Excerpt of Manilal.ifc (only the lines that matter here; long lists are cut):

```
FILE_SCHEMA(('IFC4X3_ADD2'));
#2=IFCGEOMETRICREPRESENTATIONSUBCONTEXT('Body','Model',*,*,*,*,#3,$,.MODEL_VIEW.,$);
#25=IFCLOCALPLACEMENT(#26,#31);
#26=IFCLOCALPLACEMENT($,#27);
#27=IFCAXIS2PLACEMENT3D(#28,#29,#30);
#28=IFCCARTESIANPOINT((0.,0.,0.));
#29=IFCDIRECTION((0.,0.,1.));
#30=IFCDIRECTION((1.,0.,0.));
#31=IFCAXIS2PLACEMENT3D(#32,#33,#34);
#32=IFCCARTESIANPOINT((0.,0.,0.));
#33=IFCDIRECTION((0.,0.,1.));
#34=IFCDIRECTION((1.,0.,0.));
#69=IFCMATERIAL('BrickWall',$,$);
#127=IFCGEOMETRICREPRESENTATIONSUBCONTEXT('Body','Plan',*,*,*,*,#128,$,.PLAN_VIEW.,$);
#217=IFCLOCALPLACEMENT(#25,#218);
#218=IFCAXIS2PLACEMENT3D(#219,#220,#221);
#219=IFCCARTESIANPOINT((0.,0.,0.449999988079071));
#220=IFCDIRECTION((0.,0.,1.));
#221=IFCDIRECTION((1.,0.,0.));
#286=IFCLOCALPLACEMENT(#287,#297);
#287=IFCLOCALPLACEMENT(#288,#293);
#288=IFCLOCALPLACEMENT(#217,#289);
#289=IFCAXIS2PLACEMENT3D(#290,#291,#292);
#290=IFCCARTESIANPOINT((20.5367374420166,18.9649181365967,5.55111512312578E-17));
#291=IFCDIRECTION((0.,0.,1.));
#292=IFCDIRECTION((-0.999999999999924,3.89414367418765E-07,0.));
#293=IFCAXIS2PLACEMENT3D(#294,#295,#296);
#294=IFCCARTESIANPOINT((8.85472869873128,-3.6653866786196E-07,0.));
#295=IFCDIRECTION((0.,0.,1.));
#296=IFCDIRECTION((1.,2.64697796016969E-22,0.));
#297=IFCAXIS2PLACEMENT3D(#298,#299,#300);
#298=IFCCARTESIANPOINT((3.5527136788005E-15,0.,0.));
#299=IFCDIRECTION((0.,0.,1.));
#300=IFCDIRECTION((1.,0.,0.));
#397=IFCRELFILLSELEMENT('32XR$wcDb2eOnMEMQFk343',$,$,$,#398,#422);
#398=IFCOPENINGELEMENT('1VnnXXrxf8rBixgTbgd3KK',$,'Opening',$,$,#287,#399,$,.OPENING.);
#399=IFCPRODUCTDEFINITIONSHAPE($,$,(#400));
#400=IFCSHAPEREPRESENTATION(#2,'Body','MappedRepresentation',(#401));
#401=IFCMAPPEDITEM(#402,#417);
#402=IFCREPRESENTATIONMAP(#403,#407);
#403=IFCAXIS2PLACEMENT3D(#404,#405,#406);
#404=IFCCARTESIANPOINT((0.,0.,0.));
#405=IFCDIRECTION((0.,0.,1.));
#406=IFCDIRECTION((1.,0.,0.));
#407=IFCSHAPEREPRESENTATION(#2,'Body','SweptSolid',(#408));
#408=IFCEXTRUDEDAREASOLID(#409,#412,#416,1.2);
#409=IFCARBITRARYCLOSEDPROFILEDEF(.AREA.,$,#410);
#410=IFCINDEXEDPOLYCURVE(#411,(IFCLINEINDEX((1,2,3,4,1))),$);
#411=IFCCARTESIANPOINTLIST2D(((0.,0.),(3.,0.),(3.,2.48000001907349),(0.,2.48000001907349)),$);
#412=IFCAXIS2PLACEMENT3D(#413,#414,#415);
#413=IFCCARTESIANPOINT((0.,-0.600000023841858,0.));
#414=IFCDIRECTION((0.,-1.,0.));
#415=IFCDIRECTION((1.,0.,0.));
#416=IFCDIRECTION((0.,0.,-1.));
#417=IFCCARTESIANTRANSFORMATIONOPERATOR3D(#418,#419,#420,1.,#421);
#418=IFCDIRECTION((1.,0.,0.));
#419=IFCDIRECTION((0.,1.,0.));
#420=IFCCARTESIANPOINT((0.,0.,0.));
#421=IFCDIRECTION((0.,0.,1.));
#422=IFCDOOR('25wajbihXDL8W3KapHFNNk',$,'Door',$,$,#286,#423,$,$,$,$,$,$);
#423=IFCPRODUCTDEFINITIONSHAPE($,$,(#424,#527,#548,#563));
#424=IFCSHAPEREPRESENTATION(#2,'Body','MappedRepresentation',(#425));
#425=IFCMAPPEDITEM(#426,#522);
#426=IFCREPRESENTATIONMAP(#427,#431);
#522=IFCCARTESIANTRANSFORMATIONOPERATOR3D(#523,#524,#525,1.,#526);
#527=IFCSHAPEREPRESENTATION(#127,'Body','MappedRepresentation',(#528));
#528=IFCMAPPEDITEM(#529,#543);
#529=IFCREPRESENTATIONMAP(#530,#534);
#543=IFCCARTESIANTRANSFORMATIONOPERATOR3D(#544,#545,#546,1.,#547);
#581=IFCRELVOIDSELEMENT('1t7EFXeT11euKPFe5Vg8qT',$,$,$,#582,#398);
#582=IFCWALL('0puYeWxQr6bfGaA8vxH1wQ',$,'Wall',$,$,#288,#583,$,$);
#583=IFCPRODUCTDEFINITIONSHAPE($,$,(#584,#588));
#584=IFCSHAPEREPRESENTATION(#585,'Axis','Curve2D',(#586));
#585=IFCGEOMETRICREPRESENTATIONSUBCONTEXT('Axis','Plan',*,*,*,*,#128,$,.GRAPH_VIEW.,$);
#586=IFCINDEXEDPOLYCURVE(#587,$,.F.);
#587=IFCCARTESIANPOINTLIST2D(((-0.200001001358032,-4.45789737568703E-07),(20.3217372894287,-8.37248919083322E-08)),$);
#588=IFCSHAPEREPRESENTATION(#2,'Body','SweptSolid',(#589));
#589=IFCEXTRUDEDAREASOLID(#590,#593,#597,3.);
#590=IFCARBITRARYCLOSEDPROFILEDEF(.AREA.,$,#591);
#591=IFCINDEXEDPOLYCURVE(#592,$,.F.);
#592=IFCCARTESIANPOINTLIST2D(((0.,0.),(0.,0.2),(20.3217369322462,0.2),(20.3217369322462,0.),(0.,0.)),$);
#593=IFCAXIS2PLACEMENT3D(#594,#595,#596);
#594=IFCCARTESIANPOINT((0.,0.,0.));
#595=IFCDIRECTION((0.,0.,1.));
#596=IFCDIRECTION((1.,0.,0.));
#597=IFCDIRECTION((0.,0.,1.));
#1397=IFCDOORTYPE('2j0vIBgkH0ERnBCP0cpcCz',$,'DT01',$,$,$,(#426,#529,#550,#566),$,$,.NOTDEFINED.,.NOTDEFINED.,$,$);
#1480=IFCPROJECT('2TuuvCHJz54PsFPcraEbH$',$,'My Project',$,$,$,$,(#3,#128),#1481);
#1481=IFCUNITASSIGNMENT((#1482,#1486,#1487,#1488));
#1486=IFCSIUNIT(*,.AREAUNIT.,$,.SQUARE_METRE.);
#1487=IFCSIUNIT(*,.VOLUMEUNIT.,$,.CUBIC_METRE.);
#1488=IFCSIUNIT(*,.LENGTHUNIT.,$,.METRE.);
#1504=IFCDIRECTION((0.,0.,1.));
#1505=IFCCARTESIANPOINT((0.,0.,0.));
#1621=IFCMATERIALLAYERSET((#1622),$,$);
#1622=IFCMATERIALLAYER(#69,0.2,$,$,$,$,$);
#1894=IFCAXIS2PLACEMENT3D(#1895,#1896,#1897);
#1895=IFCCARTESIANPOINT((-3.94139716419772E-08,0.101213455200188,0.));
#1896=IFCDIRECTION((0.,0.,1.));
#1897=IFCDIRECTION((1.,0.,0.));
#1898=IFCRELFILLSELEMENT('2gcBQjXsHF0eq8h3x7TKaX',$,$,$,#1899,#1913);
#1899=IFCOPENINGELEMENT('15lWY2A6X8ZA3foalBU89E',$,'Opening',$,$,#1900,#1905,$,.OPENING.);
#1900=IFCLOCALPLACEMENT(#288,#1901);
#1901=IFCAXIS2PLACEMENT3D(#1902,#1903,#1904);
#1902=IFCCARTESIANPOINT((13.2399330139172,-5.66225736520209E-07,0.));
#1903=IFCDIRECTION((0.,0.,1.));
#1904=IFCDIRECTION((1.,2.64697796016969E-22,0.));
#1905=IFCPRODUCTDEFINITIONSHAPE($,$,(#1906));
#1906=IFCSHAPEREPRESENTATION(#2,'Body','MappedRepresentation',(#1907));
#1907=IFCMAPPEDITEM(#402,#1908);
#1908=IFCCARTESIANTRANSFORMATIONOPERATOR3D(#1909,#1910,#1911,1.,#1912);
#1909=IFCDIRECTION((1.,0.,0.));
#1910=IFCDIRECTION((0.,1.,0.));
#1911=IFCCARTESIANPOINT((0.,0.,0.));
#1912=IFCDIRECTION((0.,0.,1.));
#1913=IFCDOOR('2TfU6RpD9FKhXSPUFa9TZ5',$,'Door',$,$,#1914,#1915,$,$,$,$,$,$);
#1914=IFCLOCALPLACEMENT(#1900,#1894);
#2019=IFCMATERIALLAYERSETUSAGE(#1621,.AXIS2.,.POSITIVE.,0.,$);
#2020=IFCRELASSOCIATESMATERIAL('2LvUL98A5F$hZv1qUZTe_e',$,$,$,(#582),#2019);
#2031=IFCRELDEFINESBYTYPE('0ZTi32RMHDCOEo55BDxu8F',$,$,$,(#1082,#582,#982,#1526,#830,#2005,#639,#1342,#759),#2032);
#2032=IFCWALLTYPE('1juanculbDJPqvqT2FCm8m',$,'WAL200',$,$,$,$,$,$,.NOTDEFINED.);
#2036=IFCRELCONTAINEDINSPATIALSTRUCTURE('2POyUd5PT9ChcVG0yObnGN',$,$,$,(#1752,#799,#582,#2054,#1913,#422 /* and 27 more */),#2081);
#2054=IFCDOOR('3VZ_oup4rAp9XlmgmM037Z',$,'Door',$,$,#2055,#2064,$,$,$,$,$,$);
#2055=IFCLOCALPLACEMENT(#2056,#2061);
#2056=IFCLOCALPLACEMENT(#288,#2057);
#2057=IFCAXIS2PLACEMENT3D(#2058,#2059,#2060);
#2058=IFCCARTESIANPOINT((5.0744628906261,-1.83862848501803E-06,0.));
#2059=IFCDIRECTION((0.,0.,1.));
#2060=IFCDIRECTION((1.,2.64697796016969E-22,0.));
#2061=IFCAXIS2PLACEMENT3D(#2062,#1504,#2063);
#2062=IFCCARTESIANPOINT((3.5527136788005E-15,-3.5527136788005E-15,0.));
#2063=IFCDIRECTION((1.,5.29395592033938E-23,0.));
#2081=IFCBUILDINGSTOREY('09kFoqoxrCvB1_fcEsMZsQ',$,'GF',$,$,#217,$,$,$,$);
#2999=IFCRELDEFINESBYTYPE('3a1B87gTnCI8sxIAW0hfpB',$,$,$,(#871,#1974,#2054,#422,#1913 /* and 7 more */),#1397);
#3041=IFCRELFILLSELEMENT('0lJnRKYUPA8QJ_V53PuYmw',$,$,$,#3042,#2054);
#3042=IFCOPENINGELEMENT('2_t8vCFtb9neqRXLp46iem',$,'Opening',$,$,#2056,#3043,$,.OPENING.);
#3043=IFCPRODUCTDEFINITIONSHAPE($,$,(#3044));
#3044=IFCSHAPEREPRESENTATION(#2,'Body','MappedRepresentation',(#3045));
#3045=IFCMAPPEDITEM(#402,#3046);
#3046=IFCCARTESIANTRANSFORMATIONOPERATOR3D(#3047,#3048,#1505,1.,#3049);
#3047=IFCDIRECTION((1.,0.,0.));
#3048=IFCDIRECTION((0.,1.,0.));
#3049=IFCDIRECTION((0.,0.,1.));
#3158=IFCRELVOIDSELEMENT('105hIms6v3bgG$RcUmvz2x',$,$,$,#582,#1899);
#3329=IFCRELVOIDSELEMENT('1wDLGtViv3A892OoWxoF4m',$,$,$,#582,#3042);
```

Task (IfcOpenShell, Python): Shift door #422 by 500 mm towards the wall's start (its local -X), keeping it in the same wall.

```python
import ifcopenshell
import ifcopenshell.api.geometry
import ifcopenshell.util.placement

model = ifcopenshell.open("Manilal.ifc")

door = model.by_id(422)
opening = door.FillsVoids[0].RelatingOpeningElement
wall = opening.VoidsElements[0].RelatingBuildingElement

wall_matrix = ifcopenshell.util.placement.get_local_placement(wall.ObjectPlacement)
shift = wall_matrix[:3, 0] * -0.5
before = ifcopenshell.util.placement.get_local_placement(door.ObjectPlacement)[:3, 3].copy()

# The door is placed relative to its opening, so it follows when the opening moves.
matrix = ifcopenshell.util.placement.get_local_placement(opening.ObjectPlacement)
matrix[:3, 3] += shift
ifcopenshell.api.geometry.edit_object_placement(
    model, product=opening, matrix=matrix, is_si=False, should_transform_children=True
)

after = ifcopenshell.util.placement.get_local_placement(door.ObjectPlacement)[:3, 3]
print("door moved by", (after - before).round(3) + 0.0)

model.write("Manilal_rev.ifc")
```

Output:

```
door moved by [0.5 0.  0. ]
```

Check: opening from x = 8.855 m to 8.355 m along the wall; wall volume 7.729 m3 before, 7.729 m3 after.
